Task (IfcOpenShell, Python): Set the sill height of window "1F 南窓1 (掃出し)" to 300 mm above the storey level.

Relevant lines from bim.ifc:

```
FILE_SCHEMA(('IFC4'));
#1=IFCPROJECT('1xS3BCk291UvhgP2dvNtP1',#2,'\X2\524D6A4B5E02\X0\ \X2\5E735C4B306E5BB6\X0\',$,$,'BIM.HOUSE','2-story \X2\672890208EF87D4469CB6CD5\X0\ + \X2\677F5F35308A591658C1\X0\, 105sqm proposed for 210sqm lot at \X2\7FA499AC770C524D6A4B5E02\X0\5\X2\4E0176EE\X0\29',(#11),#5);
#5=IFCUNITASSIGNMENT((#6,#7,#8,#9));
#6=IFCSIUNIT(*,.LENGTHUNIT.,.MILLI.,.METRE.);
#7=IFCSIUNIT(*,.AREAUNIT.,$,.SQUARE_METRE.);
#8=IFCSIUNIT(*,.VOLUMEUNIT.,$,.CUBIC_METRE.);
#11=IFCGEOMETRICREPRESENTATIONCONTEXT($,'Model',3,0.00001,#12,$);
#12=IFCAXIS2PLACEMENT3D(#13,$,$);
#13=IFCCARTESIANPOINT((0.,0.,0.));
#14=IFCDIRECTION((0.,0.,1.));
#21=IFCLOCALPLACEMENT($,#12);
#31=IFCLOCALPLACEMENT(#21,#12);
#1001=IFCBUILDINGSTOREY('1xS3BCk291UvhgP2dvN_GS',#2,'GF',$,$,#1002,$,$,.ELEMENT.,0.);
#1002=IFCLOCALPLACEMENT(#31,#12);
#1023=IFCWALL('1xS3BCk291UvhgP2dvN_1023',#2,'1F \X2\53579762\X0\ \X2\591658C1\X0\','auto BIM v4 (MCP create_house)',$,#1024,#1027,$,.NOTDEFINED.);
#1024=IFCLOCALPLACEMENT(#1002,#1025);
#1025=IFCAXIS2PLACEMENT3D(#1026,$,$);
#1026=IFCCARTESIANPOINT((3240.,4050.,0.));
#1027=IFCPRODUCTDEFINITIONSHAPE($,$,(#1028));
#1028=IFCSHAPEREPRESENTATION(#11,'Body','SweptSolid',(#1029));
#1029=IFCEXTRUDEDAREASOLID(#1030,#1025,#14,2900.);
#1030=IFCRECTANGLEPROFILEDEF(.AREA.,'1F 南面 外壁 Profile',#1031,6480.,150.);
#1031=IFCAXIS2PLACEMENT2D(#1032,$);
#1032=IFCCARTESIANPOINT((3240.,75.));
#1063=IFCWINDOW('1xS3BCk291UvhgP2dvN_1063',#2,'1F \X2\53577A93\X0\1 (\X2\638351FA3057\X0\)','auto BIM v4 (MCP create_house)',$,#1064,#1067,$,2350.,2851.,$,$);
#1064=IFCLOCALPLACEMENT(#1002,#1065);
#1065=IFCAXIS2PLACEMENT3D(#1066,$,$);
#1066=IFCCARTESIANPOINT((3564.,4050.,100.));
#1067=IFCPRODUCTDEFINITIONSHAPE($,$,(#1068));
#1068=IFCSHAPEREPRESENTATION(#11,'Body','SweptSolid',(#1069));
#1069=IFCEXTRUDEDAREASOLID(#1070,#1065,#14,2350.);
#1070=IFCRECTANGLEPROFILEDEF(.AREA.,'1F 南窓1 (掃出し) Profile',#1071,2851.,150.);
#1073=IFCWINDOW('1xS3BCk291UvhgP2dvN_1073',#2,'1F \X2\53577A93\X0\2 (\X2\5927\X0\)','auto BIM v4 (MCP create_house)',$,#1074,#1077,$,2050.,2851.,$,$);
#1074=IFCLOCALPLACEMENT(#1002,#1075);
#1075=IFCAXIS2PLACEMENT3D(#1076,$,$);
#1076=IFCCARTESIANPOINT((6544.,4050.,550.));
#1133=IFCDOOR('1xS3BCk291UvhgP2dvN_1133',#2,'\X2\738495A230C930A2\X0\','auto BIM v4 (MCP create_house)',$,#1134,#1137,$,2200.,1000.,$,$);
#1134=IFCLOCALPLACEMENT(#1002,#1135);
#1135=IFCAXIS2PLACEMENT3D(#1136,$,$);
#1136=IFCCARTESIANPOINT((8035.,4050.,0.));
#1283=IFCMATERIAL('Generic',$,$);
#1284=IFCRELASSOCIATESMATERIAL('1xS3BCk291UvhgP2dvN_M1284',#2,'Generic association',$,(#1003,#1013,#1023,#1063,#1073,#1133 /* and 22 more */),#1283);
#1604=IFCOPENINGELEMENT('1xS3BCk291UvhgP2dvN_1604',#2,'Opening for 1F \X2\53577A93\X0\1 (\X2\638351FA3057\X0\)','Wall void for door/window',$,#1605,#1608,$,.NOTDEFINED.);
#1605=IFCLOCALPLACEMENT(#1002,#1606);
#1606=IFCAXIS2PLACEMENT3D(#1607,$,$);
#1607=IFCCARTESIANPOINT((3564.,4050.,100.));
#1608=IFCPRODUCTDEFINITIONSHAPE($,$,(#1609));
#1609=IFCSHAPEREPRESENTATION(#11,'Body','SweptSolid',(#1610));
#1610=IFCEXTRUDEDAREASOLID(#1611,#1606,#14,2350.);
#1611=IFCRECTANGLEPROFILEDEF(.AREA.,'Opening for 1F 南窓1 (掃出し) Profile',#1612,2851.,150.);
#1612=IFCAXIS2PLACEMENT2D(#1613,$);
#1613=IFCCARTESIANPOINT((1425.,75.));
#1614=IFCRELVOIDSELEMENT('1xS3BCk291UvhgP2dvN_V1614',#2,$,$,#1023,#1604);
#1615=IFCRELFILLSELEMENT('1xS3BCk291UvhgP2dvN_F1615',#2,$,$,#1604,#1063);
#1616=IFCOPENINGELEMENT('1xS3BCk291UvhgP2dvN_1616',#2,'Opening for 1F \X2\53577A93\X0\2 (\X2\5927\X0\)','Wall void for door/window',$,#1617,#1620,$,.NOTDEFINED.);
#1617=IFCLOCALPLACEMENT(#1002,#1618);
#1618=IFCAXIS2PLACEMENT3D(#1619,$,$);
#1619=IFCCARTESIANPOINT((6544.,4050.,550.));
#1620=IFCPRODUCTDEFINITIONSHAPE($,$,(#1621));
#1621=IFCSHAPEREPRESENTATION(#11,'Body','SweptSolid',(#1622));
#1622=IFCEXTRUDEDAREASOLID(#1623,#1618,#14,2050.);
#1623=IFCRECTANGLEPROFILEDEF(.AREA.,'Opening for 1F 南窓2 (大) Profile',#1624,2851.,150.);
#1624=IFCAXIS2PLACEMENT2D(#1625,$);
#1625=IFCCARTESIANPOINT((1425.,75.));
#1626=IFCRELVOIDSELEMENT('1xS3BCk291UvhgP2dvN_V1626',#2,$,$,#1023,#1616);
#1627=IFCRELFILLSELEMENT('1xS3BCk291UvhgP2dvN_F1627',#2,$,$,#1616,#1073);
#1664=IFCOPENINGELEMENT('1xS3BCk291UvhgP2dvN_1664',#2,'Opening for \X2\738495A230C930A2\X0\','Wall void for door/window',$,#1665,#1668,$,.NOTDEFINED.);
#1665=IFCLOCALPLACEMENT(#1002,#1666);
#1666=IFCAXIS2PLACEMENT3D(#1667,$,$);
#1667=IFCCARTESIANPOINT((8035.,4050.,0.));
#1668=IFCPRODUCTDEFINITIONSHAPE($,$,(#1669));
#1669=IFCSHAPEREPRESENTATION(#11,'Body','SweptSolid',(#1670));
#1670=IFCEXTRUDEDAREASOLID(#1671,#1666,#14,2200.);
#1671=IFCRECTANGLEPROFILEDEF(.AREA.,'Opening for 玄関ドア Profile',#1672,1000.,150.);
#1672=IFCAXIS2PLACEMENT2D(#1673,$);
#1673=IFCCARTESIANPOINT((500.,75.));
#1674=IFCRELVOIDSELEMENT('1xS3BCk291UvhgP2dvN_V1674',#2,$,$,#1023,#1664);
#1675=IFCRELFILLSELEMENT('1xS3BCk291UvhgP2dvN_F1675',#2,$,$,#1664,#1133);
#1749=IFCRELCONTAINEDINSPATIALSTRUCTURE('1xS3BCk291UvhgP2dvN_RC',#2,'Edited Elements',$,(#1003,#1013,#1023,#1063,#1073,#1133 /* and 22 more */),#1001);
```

```python
import numpy as np
import ifcopenshell
import ifcopenshell.api.geometry
import ifcopenshell.geom
import ifcopenshell.util.element
import ifcopenshell.util.placement
import ifcopenshell.util.shape
import ifcopenshell.util.unit

model = ifcopenshell.open("bim.ifc")
unit_scale = ifcopenshell.util.unit.calculate_unit_scale(model)

window = model.by_guid("1xS3BCk291UvhgP2dvN_1063")
opening = window.FillsVoids[0].RelatingOpeningElement
storey = ifcopenshell.util.element.get_container(window, ifc_class="IfcBuildingStorey")
level = ifcopenshell.util.placement.get_local_placement(storey.ObjectPlacement)[2, 3]

# The opening's origin need not be at the sill, so measure its lowest point.
shape = ifcopenshell.geom.create_shape(ifcopenshell.geom.settings(), opening)
bottom = ifcopenshell.util.shape.get_shape_bottom_elevation(shape, shape.geometry) / unit_scale
dz = level + 0.3 / unit_scale - bottom

shift = np.array([0.0, 0.0, dz])
# The window is not placed relative to its opening, so move both.
for product in (opening, window):
    matrix = ifcopenshell.util.placement.get_local_placement(product.ObjectPlacement)
    matrix[:3, 3] += shift
    ifcopenshell.api.geometry.edit_object_placement(model, product=product, matrix=matrix, is_si=False)

print(f"moved by {dz * unit_scale:+.3f} m")

model.write("bim_edited.ifc")
```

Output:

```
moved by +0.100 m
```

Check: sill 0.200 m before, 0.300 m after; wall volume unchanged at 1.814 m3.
